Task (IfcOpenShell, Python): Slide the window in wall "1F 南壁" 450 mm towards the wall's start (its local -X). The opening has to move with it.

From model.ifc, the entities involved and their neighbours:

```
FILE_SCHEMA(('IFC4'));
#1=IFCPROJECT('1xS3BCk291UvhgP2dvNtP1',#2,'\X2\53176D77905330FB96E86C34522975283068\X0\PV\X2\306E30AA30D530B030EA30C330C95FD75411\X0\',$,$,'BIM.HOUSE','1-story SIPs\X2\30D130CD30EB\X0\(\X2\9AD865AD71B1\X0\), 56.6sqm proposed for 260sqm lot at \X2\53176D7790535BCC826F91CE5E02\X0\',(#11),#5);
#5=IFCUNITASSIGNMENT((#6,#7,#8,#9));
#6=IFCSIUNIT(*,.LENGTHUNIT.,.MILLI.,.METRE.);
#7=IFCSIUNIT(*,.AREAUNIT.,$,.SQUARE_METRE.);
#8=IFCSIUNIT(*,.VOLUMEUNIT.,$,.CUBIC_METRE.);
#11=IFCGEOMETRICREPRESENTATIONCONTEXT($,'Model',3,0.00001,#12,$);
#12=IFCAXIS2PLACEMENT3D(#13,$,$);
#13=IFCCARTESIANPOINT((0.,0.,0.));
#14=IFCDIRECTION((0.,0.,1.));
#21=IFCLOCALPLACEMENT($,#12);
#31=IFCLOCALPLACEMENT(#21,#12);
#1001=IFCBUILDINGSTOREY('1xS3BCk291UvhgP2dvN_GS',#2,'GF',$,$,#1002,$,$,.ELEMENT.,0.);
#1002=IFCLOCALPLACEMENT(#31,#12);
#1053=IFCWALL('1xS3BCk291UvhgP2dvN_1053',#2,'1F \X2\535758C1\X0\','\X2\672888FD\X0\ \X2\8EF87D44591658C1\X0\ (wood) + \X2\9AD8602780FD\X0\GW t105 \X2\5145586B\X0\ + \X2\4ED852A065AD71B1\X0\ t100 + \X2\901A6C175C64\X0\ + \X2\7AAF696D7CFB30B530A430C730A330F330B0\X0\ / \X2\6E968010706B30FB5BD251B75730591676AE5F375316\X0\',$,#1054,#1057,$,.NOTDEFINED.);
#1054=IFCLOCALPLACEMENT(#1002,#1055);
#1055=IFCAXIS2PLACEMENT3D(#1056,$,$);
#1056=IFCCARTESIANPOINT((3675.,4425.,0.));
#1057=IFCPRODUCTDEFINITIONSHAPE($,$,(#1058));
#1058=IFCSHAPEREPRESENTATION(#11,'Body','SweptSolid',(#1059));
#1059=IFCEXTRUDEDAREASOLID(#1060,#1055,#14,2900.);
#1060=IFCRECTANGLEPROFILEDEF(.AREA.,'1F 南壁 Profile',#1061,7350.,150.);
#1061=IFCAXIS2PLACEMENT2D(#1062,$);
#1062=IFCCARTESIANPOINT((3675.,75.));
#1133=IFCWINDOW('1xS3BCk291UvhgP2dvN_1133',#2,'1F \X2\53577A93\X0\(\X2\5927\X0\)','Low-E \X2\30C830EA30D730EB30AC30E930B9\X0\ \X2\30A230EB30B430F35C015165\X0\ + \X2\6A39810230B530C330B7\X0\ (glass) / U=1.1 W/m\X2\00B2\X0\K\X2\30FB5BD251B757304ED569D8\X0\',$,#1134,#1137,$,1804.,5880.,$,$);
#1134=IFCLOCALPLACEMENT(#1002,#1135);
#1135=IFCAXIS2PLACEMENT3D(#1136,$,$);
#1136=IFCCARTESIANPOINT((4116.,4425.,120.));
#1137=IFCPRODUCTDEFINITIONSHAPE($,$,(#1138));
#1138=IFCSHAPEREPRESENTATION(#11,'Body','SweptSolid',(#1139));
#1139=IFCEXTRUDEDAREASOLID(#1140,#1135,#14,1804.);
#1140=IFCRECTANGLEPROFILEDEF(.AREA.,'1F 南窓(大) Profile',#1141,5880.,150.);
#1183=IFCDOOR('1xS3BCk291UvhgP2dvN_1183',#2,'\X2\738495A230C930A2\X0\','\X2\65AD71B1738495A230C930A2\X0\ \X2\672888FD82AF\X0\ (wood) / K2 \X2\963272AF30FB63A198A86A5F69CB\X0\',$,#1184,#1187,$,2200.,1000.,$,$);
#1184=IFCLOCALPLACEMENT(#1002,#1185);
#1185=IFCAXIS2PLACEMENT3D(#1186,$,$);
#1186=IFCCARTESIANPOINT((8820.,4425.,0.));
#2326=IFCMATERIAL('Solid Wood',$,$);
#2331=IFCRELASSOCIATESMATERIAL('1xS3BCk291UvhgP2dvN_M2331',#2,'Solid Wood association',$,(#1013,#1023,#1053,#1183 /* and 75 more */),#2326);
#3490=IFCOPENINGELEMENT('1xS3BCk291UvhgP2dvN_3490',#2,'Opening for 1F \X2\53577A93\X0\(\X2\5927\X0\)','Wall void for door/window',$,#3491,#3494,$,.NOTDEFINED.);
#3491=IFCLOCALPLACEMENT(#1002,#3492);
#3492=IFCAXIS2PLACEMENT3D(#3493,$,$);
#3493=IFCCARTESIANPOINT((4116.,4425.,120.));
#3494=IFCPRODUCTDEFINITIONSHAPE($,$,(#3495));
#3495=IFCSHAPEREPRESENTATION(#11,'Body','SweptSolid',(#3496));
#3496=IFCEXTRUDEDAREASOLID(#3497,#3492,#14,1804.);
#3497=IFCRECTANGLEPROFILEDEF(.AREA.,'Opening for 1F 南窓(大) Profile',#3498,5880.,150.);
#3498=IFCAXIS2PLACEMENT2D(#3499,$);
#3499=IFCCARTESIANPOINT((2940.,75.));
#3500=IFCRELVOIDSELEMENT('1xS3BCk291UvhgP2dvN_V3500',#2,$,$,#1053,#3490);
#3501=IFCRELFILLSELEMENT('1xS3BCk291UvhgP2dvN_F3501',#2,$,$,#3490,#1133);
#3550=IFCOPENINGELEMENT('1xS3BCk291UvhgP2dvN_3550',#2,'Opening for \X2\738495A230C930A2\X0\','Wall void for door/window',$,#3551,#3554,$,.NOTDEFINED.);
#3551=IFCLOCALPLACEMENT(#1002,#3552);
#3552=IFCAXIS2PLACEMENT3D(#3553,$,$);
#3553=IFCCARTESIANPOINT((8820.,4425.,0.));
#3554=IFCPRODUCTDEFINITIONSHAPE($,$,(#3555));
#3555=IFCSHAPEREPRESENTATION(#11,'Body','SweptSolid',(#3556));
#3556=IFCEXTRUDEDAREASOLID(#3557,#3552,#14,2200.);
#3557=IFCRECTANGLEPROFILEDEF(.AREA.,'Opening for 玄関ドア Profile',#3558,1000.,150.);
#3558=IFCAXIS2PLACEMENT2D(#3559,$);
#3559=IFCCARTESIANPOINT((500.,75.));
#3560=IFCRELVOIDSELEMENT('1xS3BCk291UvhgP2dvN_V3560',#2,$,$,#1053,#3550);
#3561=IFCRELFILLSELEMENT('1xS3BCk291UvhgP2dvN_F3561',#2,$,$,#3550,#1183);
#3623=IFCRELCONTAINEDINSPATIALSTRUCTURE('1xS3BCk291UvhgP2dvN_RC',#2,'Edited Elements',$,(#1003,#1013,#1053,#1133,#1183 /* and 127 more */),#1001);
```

```python
import ifcopenshell
import ifcopenshell.api.geometry
import ifcopenshell.util.placement
import ifcopenshell.util.unit

model = ifcopenshell.open("model.ifc")
unit_scale = ifcopenshell.util.unit.calculate_unit_scale(model)

window = model.by_guid("1xS3BCk291UvhgP2dvN_1133")
opening = window.FillsVoids[0].RelatingOpeningElement
wall = opening.VoidsElements[0].RelatingBuildingElement

wall_matrix = ifcopenshell.util.placement.get_local_placement(wall.ObjectPlacement)
shift = wall_matrix[:3, 0] * -0.45 / unit_scale
before = ifcopenshell.util.placement.get_local_placement(window.ObjectPlacement)[:3, 3].copy()

# The window is not placed relative to its opening, so move both.
for product in (opening, window):
    matrix = ifcopenshell.util.placement.get_local_placement(product.ObjectPlacement)
    matrix[:3, 3] += shift
    ifcopenshell.api.geometry.edit_object_placement(model, product=product, matrix=matrix, is_si=False)

after = ifcopenshell.util.placement.get_local_placement(window.ObjectPlacement)[:3, 3]
print("window moved by", (after - before).round(3) + 0.0)

model.write("model_updated.ifc")
```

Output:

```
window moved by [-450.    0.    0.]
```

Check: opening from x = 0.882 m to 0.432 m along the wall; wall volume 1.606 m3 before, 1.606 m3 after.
